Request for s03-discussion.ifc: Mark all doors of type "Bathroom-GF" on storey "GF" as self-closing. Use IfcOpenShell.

First a look at what the model holds.

```python
import ifcopenshell
import ifcopenshell.util.element

model = ifcopenshell.open("s03-discussion.ifc")
print(model.schema)
storey = next(s for s in model.by_type("IfcBuildingStorey") if s.Name == "GF")
doors = [e for e in ifcopenshell.util.element.get_decomposition(storey) if e.is_a("IfcDoor")]
seen = {}
for e in doors:
    element_type = ifcopenshell.util.element.get_type(e)
    key = (element_type.Name if element_type != e and element_type else None, ifcopenshell.util.element.get_pset(e, "Pset_DoorCommon", "SelfClosing"))
    seen[key] = seen.get(key, 0) + 1
for (name, value), count in sorted(seen.items(), key=str):
    print(count, "x", name, "|", value)
```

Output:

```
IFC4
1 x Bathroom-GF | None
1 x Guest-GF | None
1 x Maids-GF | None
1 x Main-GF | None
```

```python
import ifcopenshell
import ifcopenshell.api.pset
import ifcopenshell.util.element

model = ifcopenshell.open("s03-discussion.ifc")

storey = next(s for s in model.by_type("IfcBuildingStorey") if s.Name == "GF")
doors = [e for e in ifcopenshell.util.element.get_decomposition(storey) if e.is_a("IfcDoor")]

count = 0
for e in doors:
    element_type = ifcopenshell.util.element.get_type(e)
    if element_type in (None, e) or element_type.Name != "Bathroom-GF":
        continue
    # add_pset returns the element's existing set when there is one.
    pset = ifcopenshell.api.pset.add_pset(model, product=e, name="Pset_DoorCommon")
    ifcopenshell.api.pset.edit_pset(model, pset=pset, properties={"SelfClosing": True})
    count += 1

print(count, "doors updated")

model.write("s03-discussion-out.ifc")
```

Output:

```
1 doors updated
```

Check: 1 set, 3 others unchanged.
